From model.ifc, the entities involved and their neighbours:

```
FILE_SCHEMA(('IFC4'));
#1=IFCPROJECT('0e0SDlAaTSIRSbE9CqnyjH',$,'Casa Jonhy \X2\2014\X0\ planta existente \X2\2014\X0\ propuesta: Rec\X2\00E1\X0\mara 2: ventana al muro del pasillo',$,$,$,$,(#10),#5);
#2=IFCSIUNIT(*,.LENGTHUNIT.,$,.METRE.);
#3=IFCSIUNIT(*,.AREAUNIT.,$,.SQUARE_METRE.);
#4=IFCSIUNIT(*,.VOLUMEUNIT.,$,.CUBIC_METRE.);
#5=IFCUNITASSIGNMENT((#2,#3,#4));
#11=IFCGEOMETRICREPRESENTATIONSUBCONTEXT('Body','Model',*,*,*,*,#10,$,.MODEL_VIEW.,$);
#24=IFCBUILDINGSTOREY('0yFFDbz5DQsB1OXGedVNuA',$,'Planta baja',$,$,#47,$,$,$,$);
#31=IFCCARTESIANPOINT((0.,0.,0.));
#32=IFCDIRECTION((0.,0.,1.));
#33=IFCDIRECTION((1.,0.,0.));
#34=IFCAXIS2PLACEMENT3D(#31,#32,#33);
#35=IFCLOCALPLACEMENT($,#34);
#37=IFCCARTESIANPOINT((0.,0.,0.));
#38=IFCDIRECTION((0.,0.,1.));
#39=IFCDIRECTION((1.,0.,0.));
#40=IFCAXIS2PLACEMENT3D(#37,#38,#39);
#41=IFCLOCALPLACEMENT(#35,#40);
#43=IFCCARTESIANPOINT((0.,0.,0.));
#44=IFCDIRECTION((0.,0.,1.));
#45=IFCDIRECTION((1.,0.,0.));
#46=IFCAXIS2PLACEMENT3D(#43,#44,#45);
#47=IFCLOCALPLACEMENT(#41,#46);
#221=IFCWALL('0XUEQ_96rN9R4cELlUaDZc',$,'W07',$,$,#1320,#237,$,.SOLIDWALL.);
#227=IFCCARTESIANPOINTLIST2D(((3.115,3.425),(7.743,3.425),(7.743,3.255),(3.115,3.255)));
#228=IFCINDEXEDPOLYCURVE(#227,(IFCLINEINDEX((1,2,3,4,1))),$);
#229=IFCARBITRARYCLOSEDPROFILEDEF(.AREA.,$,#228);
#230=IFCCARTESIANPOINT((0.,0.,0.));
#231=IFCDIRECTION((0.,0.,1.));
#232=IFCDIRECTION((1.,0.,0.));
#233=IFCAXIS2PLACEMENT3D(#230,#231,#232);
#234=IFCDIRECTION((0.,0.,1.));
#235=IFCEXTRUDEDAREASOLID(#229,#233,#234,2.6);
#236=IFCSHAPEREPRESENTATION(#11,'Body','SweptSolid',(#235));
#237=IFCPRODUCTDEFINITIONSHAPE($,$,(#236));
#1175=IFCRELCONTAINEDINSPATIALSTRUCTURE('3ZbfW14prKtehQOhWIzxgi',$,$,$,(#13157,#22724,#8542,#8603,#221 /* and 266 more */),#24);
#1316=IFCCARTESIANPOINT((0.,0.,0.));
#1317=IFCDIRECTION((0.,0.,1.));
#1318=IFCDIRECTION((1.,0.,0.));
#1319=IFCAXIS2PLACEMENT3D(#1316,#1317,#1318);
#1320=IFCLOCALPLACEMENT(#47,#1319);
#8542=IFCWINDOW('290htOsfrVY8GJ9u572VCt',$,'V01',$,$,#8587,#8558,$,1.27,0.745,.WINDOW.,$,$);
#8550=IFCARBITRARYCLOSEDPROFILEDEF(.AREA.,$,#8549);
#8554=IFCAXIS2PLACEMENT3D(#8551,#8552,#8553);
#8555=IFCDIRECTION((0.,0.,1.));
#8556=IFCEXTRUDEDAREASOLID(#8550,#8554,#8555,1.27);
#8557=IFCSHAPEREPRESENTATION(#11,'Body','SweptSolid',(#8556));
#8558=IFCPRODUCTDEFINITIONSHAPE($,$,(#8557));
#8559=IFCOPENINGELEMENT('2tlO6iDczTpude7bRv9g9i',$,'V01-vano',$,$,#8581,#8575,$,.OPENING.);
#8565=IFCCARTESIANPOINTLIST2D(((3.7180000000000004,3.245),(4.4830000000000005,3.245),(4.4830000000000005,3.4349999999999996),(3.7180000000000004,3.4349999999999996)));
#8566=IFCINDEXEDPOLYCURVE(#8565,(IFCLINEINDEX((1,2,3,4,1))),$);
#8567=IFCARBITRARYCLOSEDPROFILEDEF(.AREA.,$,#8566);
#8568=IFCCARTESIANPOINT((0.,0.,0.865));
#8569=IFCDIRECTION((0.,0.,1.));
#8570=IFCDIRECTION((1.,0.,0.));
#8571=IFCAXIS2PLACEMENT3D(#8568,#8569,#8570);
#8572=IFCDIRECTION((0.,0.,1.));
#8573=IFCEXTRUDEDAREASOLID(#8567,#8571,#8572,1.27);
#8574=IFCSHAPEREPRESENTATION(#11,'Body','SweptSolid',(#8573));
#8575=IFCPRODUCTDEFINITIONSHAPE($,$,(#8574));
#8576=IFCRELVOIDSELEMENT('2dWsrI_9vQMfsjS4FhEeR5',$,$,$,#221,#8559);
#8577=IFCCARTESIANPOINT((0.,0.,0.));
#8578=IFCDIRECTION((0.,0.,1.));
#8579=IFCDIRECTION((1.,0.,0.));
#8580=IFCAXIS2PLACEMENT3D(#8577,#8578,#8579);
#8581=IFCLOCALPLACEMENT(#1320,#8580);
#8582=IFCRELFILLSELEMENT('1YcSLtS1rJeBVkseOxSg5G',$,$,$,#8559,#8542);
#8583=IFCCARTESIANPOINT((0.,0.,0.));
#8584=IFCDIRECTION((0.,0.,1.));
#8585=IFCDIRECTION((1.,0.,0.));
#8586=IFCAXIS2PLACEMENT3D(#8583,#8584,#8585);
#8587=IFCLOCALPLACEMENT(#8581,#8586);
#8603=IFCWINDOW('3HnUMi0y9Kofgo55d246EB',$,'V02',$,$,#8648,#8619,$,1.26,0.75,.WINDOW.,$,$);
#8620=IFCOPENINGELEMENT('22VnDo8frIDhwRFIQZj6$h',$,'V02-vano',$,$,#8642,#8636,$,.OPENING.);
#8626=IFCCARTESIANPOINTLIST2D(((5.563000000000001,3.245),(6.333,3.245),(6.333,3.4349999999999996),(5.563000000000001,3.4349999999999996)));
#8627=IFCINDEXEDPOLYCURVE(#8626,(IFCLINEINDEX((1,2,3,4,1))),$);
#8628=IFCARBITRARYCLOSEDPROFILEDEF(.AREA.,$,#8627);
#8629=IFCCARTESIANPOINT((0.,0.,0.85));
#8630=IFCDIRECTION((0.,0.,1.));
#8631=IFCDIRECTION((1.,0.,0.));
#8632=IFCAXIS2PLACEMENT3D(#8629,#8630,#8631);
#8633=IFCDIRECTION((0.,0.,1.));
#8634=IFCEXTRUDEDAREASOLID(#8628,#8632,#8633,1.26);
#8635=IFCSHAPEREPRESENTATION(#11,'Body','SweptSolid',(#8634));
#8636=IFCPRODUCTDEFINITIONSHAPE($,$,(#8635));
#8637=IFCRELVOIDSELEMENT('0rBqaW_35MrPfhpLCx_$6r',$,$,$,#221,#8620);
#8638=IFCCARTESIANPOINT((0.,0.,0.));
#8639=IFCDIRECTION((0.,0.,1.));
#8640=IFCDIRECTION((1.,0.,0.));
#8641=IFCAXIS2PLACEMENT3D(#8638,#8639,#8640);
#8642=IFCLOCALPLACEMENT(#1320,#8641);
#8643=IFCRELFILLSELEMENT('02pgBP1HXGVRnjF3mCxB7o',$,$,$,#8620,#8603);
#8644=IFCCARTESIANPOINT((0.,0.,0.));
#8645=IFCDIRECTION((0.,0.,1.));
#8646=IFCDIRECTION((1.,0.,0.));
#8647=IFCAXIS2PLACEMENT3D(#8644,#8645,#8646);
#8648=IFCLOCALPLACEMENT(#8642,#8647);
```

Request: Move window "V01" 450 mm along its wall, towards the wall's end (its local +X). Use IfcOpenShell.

```python
import ifcopenshell
import ifcopenshell.api.geometry
import ifcopenshell.util.placement

model = ifcopenshell.open("model.ifc")

window = model.by_id(8542)
opening = window.FillsVoids[0].RelatingOpeningElement
wall = opening.VoidsElements[0].RelatingBuildingElement

wall_matrix = ifcopenshell.util.placement.get_local_placement(wall.ObjectPlacement)
shift = wall_matrix[:3, 0] * 0.45
before = ifcopenshell.util.placement.get_local_placement(window.ObjectPlacement)[:3, 3].copy()

# The window is placed relative to its opening, so it follows when the opening moves.
matrix = ifcopenshell.util.placement.get_local_placement(opening.ObjectPlacement)
matrix[:3, 3] += shift
ifcopenshell.api.geometry.edit_object_placement(
    model, product=opening, matrix=matrix, is_si=False, should_transform_children=True
)

after = ifcopenshell.util.placement.get_local_placement(window.ObjectPlacement)[:3, 3]
print("window moved by", (after - before).round(3) + 0.0)

model.write("model_v2.ifc")
```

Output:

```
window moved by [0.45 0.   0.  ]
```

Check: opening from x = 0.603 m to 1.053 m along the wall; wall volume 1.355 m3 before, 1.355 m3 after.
